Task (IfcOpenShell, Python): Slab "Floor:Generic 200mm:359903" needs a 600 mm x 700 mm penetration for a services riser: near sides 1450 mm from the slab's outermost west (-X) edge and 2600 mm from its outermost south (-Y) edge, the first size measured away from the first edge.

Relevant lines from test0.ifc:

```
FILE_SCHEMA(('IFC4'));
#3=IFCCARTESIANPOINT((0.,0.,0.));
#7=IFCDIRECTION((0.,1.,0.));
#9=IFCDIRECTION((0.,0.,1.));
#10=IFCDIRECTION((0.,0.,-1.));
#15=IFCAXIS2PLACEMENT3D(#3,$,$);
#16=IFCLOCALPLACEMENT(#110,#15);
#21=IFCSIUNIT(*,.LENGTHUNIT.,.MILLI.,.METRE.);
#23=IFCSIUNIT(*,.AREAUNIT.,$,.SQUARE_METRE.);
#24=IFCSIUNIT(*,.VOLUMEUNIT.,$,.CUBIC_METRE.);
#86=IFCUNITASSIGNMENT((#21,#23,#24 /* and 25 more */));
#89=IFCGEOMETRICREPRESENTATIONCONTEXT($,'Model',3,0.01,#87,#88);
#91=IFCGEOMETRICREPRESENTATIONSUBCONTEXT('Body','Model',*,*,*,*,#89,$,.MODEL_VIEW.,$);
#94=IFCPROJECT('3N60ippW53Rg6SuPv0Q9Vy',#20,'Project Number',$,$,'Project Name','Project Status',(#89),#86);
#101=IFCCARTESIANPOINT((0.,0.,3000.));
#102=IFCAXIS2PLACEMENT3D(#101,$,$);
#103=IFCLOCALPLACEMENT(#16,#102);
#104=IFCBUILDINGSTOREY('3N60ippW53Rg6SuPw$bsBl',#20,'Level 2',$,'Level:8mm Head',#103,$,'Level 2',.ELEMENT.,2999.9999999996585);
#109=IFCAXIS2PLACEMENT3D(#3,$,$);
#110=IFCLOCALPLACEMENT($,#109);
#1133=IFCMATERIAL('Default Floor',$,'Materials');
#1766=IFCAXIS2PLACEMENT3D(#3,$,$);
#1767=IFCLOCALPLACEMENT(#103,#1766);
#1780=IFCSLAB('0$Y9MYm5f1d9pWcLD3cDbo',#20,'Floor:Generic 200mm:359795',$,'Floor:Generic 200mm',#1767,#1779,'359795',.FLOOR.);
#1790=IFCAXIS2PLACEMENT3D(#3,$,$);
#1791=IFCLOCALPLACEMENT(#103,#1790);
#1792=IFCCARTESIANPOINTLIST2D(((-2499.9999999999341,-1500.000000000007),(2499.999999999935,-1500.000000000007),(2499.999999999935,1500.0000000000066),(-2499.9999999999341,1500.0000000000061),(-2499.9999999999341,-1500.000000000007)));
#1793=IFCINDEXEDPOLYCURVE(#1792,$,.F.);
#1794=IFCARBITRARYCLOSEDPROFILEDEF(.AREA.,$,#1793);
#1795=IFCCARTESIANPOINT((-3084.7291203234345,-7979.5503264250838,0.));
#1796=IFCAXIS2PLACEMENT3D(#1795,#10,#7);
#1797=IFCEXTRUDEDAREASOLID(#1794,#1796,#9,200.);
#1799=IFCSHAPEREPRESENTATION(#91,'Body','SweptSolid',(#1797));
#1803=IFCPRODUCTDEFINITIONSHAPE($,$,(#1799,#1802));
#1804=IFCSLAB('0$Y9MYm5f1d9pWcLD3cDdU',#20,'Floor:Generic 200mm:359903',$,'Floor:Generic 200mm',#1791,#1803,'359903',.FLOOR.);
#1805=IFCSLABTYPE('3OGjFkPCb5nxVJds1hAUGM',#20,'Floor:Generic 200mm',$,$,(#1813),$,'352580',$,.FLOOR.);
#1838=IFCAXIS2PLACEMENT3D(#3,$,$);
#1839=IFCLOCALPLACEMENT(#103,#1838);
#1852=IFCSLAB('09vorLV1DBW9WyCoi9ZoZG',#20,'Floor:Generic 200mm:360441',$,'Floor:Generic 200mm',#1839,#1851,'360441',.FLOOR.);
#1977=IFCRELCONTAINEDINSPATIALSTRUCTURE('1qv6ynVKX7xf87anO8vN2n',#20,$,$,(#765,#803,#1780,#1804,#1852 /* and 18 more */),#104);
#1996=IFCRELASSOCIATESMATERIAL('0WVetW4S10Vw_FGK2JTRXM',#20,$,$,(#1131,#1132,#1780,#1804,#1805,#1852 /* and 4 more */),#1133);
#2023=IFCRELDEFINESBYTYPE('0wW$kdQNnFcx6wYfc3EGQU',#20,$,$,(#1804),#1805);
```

```python
import numpy as np
import ifcopenshell
import ifcopenshell.api.feature
import ifcopenshell.api.geometry
import ifcopenshell.api.root
import ifcopenshell.geom
import ifcopenshell.util.placement
import ifcopenshell.util.representation
import ifcopenshell.util.shape
import ifcopenshell.util.unit

model = ifcopenshell.open("test0.ifc")
unit_scale = ifcopenshell.util.unit.calculate_unit_scale(model)
settings = ifcopenshell.geom.settings()


def volume(element):
    """Net volume in cubic metres, openings subtracted."""
    shape = ifcopenshell.geom.create_shape(settings, element)
    return ifcopenshell.util.shape.get_volume(shape.geometry)


slab = model.by_guid("0$Y9MYm5f1d9pWcLD3cDdU")
before = volume(slab)

# Extent in the slab's own axes, in metres. The edges named are its -X and -Y sides.
slab_shape = ifcopenshell.geom.create_shape(settings, slab)
vertices = ifcopenshell.util.shape.get_vertices(slab_shape.geometry)
x_min, y_min, bottom = vertices.min(axis=0)
top = vertices[:, 2].max()

opening = ifcopenshell.api.root.create_entity(model, ifc_class="IfcOpeningElement", name="Services riser opening", predefined_type="OPENING")
context = ifcopenshell.util.representation.get_context(model, "Model", "Body", "MODEL_VIEW")
width, depth = 0.6, 0.7
outline = [(0.0, 0.0), (width, 0.0), (width, depth), (0.0, depth), (0.0, 0.0)]
# Overshoot both faces by 50 mm so the cut is clean.
shape = ifcopenshell.api.geometry.add_slab_representation(
    model, context=context, depth=top - bottom + 0.1, polyline=outline
)
ifcopenshell.api.geometry.assign_representation(model, product=opening, representation=shape)

matrix = ifcopenshell.util.placement.get_local_placement(slab.ObjectPlacement)
matrix[:, 3] = matrix @ np.append(np.array([x_min + 1.45, y_min + 2.6, bottom - 0.05]) / unit_scale, 1.0)
ifcopenshell.api.geometry.edit_object_placement(model, product=opening, matrix=matrix, is_si=False)
ifcopenshell.api.feature.add_feature(model, feature=opening, element=slab)

after = volume(slab)

print(f"slab volume {before:.3f} -> {after:.3f} m3")

model.write("test0_updated.ifc")
```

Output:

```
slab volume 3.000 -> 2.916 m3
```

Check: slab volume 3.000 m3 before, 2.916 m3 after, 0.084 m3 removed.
